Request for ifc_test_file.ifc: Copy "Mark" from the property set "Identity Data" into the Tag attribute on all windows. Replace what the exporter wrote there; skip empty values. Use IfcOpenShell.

First a look at what the model holds.

```python
import ifcopenshell
import ifcopenshell.util.element

model = ifcopenshell.open("ifc_test_file.ifc")
print(model.schema)
windows = model.by_type("IfcWindow")
print(len(windows), "windows")
for e in windows[:8]:
    source = ifcopenshell.util.element.get_pset(e, "Identity Data", "Mark")
    target = e.Tag
    print(e.id(), repr(source), repr(target), sep=" | ")
```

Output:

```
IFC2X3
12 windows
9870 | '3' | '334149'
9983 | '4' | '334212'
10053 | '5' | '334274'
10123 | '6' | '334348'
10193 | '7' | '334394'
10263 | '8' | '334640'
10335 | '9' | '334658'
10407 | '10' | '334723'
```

```python
import ifcopenshell
import ifcopenshell.util.element

model = ifcopenshell.open("ifc_test_file.ifc")

count = 0
for e in model.by_type("IfcWindow"):
    value = ifcopenshell.util.element.get_pset(e, "Identity Data", "Mark")
    current = e.Tag
    if not value or not value.strip() or current == value:
        continue
    e.Tag = value
    count += 1

print(count, "windows updated")

model.write("ifc_test_file_rev.ifc")
```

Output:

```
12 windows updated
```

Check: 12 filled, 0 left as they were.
